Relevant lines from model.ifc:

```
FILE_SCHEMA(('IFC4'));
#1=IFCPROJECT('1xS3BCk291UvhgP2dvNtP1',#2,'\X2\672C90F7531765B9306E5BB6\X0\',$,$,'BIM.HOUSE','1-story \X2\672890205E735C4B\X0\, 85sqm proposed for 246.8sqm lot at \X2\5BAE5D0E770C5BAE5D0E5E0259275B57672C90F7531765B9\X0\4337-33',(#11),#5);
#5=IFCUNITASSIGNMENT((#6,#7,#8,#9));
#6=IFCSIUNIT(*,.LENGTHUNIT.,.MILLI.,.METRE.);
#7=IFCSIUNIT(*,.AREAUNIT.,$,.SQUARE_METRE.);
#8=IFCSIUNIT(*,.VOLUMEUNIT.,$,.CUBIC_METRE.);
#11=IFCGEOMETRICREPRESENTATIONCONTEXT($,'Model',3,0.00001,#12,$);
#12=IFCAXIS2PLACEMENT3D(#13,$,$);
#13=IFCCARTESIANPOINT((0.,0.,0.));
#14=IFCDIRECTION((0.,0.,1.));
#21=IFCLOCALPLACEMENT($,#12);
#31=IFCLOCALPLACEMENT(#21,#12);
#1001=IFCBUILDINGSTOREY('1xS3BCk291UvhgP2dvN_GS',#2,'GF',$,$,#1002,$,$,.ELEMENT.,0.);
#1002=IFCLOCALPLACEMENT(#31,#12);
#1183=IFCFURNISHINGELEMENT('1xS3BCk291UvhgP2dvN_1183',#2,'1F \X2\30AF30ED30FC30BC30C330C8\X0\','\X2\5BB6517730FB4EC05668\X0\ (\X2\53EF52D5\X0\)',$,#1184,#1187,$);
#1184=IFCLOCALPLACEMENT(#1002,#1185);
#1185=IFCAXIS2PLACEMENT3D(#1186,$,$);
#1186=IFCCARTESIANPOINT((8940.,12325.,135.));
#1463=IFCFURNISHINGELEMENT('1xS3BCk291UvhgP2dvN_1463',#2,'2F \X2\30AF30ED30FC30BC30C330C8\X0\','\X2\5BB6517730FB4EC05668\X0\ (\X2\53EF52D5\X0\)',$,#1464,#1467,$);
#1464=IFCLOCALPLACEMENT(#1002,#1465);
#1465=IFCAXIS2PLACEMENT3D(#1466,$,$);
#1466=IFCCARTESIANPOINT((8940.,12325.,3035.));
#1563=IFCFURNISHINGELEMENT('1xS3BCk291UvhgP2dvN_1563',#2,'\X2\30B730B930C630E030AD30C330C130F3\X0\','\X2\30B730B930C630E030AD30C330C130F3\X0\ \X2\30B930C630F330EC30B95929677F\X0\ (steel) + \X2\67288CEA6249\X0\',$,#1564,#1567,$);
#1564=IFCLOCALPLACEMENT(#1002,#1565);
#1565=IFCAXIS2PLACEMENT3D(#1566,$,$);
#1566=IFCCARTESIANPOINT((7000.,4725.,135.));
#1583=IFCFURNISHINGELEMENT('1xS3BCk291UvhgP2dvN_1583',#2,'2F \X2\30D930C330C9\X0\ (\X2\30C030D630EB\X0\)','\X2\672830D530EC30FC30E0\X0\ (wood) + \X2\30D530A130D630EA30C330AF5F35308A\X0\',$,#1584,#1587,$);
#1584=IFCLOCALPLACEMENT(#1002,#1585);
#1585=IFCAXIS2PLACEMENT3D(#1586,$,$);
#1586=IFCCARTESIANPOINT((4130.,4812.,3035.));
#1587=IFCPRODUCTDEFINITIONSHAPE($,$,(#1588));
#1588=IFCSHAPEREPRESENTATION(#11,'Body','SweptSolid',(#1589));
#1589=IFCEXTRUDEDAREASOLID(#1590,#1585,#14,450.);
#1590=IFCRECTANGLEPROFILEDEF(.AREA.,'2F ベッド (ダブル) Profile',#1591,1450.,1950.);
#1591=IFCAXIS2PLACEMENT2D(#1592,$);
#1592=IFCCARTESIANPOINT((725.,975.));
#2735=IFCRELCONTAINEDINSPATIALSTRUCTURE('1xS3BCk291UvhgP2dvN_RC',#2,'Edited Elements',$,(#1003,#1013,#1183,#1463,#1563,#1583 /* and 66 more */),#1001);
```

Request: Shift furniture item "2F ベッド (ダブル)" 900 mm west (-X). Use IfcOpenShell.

```python
import ifcopenshell
import ifcopenshell.api.geometry
import ifcopenshell.util.placement

model = ifcopenshell.open("model.ifc")

item = model.by_guid("1xS3BCk291UvhgP2dvN_1583")
matrix = ifcopenshell.util.placement.get_local_placement(item.ObjectPlacement)
matrix[0, 3] -= 900.0
ifcopenshell.api.geometry.edit_object_placement(model, product=item, matrix=matrix, is_si=False)

print(ifcopenshell.util.placement.get_local_placement(item.ObjectPlacement).round(3) + 0.0)

model.write("model_rev.ifc")
```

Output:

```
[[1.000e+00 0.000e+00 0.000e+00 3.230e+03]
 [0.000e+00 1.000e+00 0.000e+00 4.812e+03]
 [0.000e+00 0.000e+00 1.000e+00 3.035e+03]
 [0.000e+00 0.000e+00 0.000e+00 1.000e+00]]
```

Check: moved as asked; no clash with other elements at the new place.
